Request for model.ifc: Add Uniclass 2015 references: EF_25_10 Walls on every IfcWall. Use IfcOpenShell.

First a look at what the model holds.

```python
import ifcopenshell

model = ifcopenshell.open("model.ifc")
print(model.schema)
print("classifications:", [c.Name for c in model.by_type("IfcClassification")])
for ifc_class in ("IfcDoor", "IfcRoof", "IfcStair", "IfcWall", "IfcWindow"):
    print(ifc_class, len(model.by_type(ifc_class)))
```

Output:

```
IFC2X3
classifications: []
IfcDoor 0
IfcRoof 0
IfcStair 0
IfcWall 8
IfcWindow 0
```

```python
import ifcopenshell
import ifcopenshell.api.classification

model = ifcopenshell.open("model.ifc")

# IFC2X3 requires Source and Edition and has no link from the project to the system.
system = model.create_entity("IfcClassification", Source="NBS", Edition="2015", Name="Uniclass 2015")

codes = {
    "IfcWall": ("EF_25_10", "Walls"),
}
for ifc_class, (code, name) in codes.items():
    products = model.by_type(ifc_class)
    ifcopenshell.api.classification.add_reference(
        model, products=products, classification=system, identification=code, name=name
    )
    print(code, len(products))

model.write("model_rev.ifc")
```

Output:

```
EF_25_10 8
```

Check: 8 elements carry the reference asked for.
